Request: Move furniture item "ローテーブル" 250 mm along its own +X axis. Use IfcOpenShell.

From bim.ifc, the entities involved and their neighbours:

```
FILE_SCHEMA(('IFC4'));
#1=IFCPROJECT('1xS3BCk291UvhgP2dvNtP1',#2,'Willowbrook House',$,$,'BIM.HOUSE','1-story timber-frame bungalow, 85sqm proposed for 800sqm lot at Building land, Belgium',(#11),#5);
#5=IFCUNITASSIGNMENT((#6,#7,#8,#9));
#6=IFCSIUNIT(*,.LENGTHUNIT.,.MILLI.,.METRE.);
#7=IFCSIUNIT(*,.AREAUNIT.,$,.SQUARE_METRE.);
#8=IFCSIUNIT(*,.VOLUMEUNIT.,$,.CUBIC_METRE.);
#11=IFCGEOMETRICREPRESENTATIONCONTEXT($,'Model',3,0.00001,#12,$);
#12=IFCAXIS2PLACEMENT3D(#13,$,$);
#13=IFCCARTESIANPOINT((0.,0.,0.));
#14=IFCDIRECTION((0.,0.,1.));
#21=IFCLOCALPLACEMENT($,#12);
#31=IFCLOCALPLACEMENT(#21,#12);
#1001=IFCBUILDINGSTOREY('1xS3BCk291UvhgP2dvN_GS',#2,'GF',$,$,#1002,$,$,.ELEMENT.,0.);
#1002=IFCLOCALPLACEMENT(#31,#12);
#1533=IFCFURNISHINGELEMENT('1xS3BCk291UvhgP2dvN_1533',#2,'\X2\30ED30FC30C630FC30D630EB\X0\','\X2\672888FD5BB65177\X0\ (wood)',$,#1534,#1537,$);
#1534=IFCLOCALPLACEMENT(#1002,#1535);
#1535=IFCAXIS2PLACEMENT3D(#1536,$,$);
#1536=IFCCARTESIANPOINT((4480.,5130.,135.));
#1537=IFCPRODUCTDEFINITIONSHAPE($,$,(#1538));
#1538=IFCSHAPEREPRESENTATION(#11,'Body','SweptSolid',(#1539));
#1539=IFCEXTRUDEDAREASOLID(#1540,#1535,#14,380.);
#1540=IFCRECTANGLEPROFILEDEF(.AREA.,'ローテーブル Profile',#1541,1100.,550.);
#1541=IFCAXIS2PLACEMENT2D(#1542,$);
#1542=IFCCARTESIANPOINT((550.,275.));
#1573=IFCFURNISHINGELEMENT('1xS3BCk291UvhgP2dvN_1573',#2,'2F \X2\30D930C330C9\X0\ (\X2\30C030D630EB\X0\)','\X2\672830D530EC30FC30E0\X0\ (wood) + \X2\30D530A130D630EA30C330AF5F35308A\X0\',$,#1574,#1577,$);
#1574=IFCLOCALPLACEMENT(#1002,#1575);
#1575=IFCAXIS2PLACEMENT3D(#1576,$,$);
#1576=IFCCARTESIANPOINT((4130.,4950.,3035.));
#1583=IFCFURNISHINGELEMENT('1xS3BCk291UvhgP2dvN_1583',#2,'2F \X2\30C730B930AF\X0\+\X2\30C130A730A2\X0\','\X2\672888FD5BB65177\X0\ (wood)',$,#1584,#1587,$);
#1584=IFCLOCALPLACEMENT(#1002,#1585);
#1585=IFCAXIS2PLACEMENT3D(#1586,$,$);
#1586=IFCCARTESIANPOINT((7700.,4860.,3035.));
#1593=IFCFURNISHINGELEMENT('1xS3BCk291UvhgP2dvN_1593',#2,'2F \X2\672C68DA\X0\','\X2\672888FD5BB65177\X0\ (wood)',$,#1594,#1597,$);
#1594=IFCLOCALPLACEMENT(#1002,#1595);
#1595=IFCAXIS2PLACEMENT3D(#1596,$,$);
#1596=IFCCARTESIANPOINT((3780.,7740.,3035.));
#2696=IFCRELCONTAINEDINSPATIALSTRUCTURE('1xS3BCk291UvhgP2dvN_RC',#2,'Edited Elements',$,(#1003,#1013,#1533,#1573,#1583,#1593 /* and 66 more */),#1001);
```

```python
import ifcopenshell
import ifcopenshell.api.geometry
import ifcopenshell.util.placement
import ifcopenshell.util.unit

model = ifcopenshell.open("bim.ifc")
unit_scale = ifcopenshell.util.unit.calculate_unit_scale(model)

item = model.by_id(1533)
matrix = ifcopenshell.util.placement.get_local_placement(item.ObjectPlacement)
matrix[:3, 3] += matrix[:3, 0] * 0.25 / unit_scale
ifcopenshell.api.geometry.edit_object_placement(model, product=item, matrix=matrix, is_si=False)

print(ifcopenshell.util.placement.get_local_placement(item.ObjectPlacement).round(3) + 0.0)

model.write("bim_rev.ifc")
```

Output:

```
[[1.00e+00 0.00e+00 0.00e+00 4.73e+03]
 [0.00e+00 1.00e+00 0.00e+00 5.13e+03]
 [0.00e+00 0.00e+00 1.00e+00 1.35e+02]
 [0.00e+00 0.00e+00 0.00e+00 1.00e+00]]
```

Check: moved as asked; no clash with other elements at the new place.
